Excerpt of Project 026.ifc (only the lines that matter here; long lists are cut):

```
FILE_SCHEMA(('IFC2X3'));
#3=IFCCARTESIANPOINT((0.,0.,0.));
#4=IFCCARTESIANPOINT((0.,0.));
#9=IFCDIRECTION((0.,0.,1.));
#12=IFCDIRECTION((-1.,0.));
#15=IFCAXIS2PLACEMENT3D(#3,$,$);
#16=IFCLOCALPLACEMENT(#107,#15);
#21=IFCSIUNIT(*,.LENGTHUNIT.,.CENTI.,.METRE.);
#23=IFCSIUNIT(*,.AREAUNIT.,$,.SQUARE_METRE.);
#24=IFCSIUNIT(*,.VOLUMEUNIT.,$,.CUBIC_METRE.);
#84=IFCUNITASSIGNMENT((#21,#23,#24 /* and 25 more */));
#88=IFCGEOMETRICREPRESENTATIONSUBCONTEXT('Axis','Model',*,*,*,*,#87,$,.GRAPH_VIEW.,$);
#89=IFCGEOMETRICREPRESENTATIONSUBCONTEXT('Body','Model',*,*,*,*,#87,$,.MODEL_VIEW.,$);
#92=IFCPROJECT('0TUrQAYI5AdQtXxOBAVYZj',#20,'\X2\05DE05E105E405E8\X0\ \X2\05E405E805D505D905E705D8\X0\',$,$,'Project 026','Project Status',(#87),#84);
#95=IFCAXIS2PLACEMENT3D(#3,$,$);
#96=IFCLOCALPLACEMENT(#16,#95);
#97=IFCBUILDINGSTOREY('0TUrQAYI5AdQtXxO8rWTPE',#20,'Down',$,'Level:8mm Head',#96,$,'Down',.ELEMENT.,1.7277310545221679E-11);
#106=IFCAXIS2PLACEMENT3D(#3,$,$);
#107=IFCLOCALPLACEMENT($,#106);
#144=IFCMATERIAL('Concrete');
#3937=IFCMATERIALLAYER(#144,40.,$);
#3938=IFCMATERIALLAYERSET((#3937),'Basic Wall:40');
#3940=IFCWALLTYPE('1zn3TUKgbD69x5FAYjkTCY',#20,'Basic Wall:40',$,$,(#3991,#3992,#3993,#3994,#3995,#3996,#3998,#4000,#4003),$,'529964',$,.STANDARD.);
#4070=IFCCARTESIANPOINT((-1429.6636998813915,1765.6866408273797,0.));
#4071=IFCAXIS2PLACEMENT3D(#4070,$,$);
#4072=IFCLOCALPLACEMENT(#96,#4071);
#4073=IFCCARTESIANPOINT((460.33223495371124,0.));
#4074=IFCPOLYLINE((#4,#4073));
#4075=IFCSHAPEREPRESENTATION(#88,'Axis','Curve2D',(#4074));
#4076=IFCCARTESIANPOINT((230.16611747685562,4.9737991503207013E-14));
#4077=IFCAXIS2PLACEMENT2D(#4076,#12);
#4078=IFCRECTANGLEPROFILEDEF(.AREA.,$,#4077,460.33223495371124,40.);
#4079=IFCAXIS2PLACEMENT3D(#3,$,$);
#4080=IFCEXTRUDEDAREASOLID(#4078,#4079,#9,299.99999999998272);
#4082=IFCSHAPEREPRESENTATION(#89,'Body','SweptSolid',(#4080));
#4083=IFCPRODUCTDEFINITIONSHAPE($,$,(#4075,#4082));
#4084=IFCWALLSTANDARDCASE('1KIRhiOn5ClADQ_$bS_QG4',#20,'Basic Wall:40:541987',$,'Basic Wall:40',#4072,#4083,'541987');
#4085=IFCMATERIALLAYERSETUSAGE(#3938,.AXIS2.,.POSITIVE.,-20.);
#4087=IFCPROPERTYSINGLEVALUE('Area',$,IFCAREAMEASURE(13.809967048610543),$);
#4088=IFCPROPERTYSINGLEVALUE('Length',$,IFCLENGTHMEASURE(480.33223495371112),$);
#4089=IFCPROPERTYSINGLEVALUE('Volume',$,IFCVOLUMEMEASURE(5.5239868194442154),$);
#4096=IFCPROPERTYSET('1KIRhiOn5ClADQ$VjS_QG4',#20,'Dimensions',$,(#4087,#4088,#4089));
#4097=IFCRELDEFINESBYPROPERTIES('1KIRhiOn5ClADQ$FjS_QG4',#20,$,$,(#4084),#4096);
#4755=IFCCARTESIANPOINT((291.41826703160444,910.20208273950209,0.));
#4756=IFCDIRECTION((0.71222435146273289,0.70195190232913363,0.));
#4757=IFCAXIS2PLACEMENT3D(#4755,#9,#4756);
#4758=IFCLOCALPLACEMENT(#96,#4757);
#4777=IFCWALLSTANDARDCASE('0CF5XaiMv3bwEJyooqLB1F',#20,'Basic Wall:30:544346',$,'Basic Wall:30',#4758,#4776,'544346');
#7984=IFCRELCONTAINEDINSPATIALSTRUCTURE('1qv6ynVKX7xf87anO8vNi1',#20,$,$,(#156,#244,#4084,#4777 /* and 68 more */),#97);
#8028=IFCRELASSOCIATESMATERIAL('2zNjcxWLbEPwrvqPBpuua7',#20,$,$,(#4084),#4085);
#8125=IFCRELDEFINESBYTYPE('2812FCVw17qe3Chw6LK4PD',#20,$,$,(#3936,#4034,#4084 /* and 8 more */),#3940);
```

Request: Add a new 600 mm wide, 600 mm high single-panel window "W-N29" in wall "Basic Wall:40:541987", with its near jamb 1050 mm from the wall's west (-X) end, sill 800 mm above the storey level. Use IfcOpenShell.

```python
import numpy as np
import ifcopenshell
import ifcopenshell.api.feature
import ifcopenshell.api.geometry
import ifcopenshell.api.pset
import ifcopenshell.api.root
import ifcopenshell.api.spatial
import ifcopenshell.api.type
import ifcopenshell.geom
import ifcopenshell.util.element
import ifcopenshell.util.placement
import ifcopenshell.util.representation
import ifcopenshell.util.shape
import ifcopenshell.util.unit

model = ifcopenshell.open("Project 026.ifc")
unit_scale = ifcopenshell.util.unit.calculate_unit_scale(model)
area_scale = ifcopenshell.util.unit.calculate_unit_scale(model, "AREAUNIT")
volume_scale = ifcopenshell.util.unit.calculate_unit_scale(model, "VOLUMEUNIT")
settings = ifcopenshell.geom.settings()


def volume(element):
    """Net volume in cubic metres, openings subtracted."""
    shape = ifcopenshell.geom.create_shape(settings, element)
    return ifcopenshell.util.shape.get_volume(shape.geometry)


wall = model.by_guid("1KIRhiOn5ClADQ_$bS_QG4")
storey = ifcopenshell.util.element.get_container(wall, ifc_class="IfcBuildingStorey")
context = ifcopenshell.util.representation.get_context(model, "Model", "Body", "MODEL_VIEW")
before = volume(wall)

width, height, from_end, sill = 0.6, 0.6, 1.05, 0.8  # metres

# The wall runs along its own X axis, and the end named is its -X end.
wall_shape = ifcopenshell.geom.create_shape(settings, wall)
x, y, z = ifcopenshell.util.shape.get_vertices(wall_shape.geometry).T
start = x.min() + from_end
face, thickness = float(y.min()), float(y.max() - y.min())
wall_matrix = ifcopenshell.util.placement.get_local_placement(wall.ObjectPlacement)
level = ifcopenshell.util.placement.get_local_placement(storey.ObjectPlacement)[2, 3]


def in_wall(x, y):
    """Placement at x, y metres in the wall's axes, at sill height."""
    matrix = wall_matrix.copy()
    matrix[:, 3] = wall_matrix @ np.array([x / unit_scale, y / unit_scale, 0.0, 1.0])
    matrix[2, 3] = level + sill / unit_scale
    return matrix


# Opening: a box that overshoots both wall faces by 50 mm.
opening = ifcopenshell.api.root.create_entity(model, ifc_class="IfcOpeningElement")
box = ifcopenshell.api.geometry.add_wall_representation(
    model, context=context, length=width, height=height, thickness=thickness + 0.1
)
ifcopenshell.api.geometry.assign_representation(model, product=opening, representation=box)
ifcopenshell.api.geometry.edit_object_placement(model, product=opening, matrix=in_wall(start, face - 0.05), is_si=False)
ifcopenshell.api.feature.add_feature(model, feature=opening, element=wall)

window = ifcopenshell.api.root.create_entity(model, ifc_class="IfcWindow", name="W-N29")
window.OverallWidth, window.OverallHeight = width / unit_scale, height / unit_scale
body = ifcopenshell.api.geometry.add_window_representation(
    model,
    context=context,
    overall_width=window.OverallWidth,
    overall_height=window.OverallHeight,
    partition_type="SINGLE_PANEL",
)
ifcopenshell.api.geometry.assign_representation(model, product=window, representation=body)
ifcopenshell.api.spatial.assign_container(model, products=[window], relating_structure=storey)
fills = ifcopenshell.api.feature.add_filling(model, opening=opening, element=window)
fills.OwnerHistory = window.OwnerHistory  # required in IFC2X3

# IFC2X3 keeps the operation on the window style.
style = ifcopenshell.api.root.create_entity(model, ifc_class="IfcWindowStyle", name="W-N29")
style.OperationType, style.ConstructionType = "SINGLE_PANEL", "NOTDEFINED"
style.ParameterTakesPrecedence = style.Sizeable = False
ifcopenshell.api.type.assign_type(model, related_objects=[window], relating_type=style)

# Centre the window in the wall's thickness.
ifcopenshell.api.geometry.edit_object_placement(model, product=window, matrix=in_wall(start, face), is_si=False)
window_shape = ifcopenshell.geom.create_shape(settings, window)
depth = ifcopenshell.util.shape.get_vertices(window_shape.geometry)[:, 1]
offset = face + thickness / 2 - (depth.min() + depth.max()) / 2
ifcopenshell.api.geometry.edit_object_placement(model, product=window, matrix=in_wall(start, offset), is_si=False)

after = volume(wall)

# Update the wall's stored quantities.
pset = model.by_id(ifcopenshell.util.element.get_pset(wall, "Dimensions", should_inherit=False)["id"])
ifcopenshell.api.pset.edit_pset(model, pset=pset, properties={
    "Area": model.create_entity("IfcAreaMeasure", after / thickness / area_scale),
    "Volume": model.create_entity("IfcVolumeMeasure", after / volume_scale),
})

print(f"wall volume {before:.3f} -> {after:.3f} m3")

model.write("Project 026_v2.ifc")
```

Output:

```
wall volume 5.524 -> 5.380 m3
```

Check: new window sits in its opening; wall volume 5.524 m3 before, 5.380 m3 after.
